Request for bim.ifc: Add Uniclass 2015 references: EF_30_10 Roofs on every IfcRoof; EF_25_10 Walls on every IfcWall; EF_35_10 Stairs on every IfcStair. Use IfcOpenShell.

First a look at what the model holds.

```python
import ifcopenshell

model = ifcopenshell.open("bim.ifc")
print(model.schema)
print("classifications:", [c.Name for c in model.by_type("IfcClassification")])
for ifc_class in ("IfcDoor", "IfcRoof", "IfcStair", "IfcWall", "IfcWindow"):
    print(ifc_class, len(model.by_type(ifc_class)))
```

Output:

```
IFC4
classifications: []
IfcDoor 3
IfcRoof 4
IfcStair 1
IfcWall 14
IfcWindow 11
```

```python
import ifcopenshell
import ifcopenshell.api.classification

model = ifcopenshell.open("bim.ifc")

system = ifcopenshell.api.classification.add_classification(model, classification="Uniclass 2015")

codes = {
    "IfcRoof": ("EF_30_10", "Roofs"),
    "IfcWall": ("EF_25_10", "Walls"),
    "IfcStair": ("EF_35_10", "Stairs"),
}
for ifc_class, (code, name) in codes.items():
    products = model.by_type(ifc_class)
    ifcopenshell.api.classification.add_reference(
        model, products=products, classification=system, identification=code, name=name
    )
    print(code, len(products))

model.write("bim_v2.ifc")
```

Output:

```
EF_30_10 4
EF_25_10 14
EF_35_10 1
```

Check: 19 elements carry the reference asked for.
